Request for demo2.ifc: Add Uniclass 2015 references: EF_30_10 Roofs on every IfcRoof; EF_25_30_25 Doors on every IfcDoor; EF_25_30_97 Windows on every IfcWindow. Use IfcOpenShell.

First a look at what the model holds.

```python
import ifcopenshell

model = ifcopenshell.open("demo2.ifc")
print(model.schema)
print("classifications:", [c.Name for c in model.by_type("IfcClassification")])
for ifc_class in ("IfcDoor", "IfcRoof", "IfcStair", "IfcWall", "IfcWindow"):
    print(ifc_class, len(model.by_type(ifc_class)))
```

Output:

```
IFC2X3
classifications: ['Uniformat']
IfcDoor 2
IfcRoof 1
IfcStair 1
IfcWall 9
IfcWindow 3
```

```python
import ifcopenshell
import ifcopenshell.api.classification

model = ifcopenshell.open("demo2.ifc")

# IFC2X3 requires Source and Edition and has no link from the project to the system.
system = model.create_entity("IfcClassification", Source="NBS", Edition="2015", Name="Uniclass 2015")

codes = {
    "IfcRoof": ("EF_30_10", "Roofs"),
    "IfcDoor": ("EF_25_30_25", "Doors"),
    "IfcWindow": ("EF_25_30_97", "Windows"),
}
for ifc_class, (code, name) in codes.items():
    products = model.by_type(ifc_class)
    ifcopenshell.api.classification.add_reference(
        model, products=products, classification=system, identification=code, name=name
    )
    print(code, len(products))

model.write("demo2_updated.ifc")
```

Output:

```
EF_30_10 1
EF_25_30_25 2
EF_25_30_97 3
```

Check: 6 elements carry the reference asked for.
